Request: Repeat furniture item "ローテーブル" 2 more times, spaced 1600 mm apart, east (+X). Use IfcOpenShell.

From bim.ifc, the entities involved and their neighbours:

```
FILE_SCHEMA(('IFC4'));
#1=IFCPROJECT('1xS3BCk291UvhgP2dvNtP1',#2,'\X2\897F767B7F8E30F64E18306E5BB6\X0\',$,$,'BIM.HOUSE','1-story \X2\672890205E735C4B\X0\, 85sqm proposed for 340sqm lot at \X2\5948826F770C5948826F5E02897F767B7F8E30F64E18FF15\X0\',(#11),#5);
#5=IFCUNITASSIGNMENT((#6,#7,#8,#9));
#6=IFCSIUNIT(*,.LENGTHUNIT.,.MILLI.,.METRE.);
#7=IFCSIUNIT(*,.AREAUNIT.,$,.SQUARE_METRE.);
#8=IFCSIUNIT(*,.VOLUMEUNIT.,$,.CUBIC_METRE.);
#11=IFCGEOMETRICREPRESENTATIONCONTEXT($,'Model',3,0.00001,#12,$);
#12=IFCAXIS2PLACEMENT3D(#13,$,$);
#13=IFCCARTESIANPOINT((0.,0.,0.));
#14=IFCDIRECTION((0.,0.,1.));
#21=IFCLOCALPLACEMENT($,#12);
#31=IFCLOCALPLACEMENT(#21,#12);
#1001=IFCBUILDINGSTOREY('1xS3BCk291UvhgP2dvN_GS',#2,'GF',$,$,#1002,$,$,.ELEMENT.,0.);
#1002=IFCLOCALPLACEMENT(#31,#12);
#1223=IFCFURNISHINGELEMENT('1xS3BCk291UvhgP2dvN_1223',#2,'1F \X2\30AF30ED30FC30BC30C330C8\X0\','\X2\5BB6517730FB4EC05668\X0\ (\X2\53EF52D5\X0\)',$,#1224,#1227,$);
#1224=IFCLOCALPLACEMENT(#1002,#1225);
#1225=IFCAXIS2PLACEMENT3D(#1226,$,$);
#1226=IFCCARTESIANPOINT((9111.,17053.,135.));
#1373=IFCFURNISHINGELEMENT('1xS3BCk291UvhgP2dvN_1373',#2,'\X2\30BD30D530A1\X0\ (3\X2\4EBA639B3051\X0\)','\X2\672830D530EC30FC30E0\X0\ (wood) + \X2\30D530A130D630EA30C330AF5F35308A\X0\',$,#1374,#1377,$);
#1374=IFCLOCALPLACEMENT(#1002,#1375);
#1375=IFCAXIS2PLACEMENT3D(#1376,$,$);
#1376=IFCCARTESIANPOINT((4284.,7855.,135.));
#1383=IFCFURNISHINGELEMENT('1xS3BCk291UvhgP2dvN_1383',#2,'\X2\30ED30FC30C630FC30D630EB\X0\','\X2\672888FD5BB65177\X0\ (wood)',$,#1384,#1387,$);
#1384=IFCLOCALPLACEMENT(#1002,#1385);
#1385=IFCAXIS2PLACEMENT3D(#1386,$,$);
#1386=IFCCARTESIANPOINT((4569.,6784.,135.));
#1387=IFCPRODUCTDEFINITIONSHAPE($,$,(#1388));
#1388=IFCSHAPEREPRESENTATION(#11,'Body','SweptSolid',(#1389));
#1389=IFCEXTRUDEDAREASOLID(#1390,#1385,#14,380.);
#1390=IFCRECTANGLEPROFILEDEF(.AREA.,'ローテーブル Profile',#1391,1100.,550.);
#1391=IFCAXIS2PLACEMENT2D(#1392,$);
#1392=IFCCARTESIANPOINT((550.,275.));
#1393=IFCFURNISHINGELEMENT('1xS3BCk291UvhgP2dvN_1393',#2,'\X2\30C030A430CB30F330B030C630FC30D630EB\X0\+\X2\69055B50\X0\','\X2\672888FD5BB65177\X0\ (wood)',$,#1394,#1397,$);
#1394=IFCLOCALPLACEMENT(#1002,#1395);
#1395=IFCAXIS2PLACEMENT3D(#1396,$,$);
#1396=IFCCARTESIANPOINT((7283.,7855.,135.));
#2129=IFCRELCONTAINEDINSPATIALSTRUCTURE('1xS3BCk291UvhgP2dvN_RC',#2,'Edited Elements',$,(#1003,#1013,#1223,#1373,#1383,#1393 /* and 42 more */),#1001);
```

```python
import numpy as np
import ifcopenshell
import ifcopenshell.api.geometry
import ifcopenshell.api.root
import ifcopenshell.util.element
import ifcopenshell.util.placement
import ifcopenshell.util.unit

model = ifcopenshell.open("bim.ifc")
unit_scale = ifcopenshell.util.unit.calculate_unit_scale(model)


def reuse_history(source, copy):
    """copy_class also copies each property set's owner history, people and application; keep the originals."""
    for rel in copy.IsDefinedBy:
        if rel.is_a("IfcRelDefinesByProperties") and (history := rel.RelatingPropertyDefinition.OwnerHistory):
            rel.RelatingPropertyDefinition.OwnerHistory = source.OwnerHistory
            ifcopenshell.util.element.remove_deep2(model, history)


source = model.by_id(1383)
base = ifcopenshell.util.placement.get_local_placement(source.ObjectPlacement)
step = np.array([1.0, 0.0, 0.0]) * 1.6 / unit_scale

for i in range(1, 3):
    copy = ifcopenshell.api.root.copy_class(model, product=source)
    copy.Representation = ifcopenshell.util.element.copy_deep(
        model, source.Representation, exclude=["IfcGeometricRepresentationContext", "IfcRepresentationMap"]
    )
    reuse_history(source, copy)
    matrix = base.copy()
    matrix[:3, 3] += i * step
    print("added at", matrix[:3, 3].round(3) + 0.0)
    ifcopenshell.api.geometry.edit_object_placement(model, product=copy, matrix=matrix, is_si=False)

model.write("bim-out.ifc")
```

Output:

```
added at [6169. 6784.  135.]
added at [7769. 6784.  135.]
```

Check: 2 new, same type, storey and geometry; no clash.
